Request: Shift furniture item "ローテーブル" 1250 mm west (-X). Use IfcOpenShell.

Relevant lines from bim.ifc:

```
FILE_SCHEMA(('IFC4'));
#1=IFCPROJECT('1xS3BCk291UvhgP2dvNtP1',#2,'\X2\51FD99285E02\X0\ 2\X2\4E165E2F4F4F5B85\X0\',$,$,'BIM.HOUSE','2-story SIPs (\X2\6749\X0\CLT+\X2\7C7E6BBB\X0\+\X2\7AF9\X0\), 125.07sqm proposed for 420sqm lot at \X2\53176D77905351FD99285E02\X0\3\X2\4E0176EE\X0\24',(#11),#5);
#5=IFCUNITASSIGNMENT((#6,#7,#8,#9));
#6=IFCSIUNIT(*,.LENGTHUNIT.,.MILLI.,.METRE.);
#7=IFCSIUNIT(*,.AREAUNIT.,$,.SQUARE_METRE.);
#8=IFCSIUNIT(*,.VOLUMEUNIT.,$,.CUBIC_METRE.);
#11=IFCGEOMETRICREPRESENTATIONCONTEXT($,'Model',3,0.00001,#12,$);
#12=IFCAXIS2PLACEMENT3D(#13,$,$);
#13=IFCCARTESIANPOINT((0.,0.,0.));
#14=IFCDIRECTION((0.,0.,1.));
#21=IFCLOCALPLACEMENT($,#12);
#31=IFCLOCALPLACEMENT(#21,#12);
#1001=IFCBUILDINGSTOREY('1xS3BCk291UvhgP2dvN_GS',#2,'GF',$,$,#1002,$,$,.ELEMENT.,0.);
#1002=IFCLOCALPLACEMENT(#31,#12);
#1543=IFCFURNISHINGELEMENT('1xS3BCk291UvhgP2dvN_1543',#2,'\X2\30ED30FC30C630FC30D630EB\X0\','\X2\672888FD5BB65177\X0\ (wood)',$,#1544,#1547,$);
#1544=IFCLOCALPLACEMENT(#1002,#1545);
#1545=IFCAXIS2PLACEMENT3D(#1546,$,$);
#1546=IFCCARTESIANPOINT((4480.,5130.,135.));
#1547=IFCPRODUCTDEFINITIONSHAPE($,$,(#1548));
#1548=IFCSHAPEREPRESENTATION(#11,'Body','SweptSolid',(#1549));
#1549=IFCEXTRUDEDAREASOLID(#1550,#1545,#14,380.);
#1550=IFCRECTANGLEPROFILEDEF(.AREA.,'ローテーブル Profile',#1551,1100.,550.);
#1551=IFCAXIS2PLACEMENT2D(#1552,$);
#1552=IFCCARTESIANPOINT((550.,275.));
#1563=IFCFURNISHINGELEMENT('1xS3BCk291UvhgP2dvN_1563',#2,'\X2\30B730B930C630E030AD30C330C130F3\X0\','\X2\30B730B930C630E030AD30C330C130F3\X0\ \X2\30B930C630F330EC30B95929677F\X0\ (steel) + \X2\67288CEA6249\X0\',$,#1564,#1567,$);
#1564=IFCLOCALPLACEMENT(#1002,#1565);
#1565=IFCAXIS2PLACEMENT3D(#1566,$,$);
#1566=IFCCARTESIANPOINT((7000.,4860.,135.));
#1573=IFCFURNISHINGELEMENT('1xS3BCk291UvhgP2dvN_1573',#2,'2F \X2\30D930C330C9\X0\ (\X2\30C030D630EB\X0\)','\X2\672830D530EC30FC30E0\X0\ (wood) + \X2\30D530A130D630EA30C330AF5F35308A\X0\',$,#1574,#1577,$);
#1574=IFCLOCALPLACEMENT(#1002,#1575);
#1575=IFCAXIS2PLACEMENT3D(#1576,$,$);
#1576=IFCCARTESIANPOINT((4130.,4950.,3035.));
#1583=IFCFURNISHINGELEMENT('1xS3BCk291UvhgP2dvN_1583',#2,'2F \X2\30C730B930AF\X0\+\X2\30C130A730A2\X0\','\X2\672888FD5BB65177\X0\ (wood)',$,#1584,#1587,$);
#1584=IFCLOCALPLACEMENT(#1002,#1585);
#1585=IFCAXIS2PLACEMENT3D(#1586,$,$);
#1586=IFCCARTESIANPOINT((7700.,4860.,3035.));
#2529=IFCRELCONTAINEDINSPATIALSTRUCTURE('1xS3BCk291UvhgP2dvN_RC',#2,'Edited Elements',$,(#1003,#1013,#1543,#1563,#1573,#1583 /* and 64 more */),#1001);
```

```python
import ifcopenshell
import ifcopenshell.api.geometry
import ifcopenshell.util.placement

model = ifcopenshell.open("bim.ifc")

item = model.by_guid("1xS3BCk291UvhgP2dvN_1543")
matrix = ifcopenshell.util.placement.get_local_placement(item.ObjectPlacement)
matrix[0, 3] -= 1250.0
ifcopenshell.api.geometry.edit_object_placement(model, product=item, matrix=matrix, is_si=False)

print(ifcopenshell.util.placement.get_local_placement(item.ObjectPlacement).round(3) + 0.0)

model.write("bim_edited.ifc")
```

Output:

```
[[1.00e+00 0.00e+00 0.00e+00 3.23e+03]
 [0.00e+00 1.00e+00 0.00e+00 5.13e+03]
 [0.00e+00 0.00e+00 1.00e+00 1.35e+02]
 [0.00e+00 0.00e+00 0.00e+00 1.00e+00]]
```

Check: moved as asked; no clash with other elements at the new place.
